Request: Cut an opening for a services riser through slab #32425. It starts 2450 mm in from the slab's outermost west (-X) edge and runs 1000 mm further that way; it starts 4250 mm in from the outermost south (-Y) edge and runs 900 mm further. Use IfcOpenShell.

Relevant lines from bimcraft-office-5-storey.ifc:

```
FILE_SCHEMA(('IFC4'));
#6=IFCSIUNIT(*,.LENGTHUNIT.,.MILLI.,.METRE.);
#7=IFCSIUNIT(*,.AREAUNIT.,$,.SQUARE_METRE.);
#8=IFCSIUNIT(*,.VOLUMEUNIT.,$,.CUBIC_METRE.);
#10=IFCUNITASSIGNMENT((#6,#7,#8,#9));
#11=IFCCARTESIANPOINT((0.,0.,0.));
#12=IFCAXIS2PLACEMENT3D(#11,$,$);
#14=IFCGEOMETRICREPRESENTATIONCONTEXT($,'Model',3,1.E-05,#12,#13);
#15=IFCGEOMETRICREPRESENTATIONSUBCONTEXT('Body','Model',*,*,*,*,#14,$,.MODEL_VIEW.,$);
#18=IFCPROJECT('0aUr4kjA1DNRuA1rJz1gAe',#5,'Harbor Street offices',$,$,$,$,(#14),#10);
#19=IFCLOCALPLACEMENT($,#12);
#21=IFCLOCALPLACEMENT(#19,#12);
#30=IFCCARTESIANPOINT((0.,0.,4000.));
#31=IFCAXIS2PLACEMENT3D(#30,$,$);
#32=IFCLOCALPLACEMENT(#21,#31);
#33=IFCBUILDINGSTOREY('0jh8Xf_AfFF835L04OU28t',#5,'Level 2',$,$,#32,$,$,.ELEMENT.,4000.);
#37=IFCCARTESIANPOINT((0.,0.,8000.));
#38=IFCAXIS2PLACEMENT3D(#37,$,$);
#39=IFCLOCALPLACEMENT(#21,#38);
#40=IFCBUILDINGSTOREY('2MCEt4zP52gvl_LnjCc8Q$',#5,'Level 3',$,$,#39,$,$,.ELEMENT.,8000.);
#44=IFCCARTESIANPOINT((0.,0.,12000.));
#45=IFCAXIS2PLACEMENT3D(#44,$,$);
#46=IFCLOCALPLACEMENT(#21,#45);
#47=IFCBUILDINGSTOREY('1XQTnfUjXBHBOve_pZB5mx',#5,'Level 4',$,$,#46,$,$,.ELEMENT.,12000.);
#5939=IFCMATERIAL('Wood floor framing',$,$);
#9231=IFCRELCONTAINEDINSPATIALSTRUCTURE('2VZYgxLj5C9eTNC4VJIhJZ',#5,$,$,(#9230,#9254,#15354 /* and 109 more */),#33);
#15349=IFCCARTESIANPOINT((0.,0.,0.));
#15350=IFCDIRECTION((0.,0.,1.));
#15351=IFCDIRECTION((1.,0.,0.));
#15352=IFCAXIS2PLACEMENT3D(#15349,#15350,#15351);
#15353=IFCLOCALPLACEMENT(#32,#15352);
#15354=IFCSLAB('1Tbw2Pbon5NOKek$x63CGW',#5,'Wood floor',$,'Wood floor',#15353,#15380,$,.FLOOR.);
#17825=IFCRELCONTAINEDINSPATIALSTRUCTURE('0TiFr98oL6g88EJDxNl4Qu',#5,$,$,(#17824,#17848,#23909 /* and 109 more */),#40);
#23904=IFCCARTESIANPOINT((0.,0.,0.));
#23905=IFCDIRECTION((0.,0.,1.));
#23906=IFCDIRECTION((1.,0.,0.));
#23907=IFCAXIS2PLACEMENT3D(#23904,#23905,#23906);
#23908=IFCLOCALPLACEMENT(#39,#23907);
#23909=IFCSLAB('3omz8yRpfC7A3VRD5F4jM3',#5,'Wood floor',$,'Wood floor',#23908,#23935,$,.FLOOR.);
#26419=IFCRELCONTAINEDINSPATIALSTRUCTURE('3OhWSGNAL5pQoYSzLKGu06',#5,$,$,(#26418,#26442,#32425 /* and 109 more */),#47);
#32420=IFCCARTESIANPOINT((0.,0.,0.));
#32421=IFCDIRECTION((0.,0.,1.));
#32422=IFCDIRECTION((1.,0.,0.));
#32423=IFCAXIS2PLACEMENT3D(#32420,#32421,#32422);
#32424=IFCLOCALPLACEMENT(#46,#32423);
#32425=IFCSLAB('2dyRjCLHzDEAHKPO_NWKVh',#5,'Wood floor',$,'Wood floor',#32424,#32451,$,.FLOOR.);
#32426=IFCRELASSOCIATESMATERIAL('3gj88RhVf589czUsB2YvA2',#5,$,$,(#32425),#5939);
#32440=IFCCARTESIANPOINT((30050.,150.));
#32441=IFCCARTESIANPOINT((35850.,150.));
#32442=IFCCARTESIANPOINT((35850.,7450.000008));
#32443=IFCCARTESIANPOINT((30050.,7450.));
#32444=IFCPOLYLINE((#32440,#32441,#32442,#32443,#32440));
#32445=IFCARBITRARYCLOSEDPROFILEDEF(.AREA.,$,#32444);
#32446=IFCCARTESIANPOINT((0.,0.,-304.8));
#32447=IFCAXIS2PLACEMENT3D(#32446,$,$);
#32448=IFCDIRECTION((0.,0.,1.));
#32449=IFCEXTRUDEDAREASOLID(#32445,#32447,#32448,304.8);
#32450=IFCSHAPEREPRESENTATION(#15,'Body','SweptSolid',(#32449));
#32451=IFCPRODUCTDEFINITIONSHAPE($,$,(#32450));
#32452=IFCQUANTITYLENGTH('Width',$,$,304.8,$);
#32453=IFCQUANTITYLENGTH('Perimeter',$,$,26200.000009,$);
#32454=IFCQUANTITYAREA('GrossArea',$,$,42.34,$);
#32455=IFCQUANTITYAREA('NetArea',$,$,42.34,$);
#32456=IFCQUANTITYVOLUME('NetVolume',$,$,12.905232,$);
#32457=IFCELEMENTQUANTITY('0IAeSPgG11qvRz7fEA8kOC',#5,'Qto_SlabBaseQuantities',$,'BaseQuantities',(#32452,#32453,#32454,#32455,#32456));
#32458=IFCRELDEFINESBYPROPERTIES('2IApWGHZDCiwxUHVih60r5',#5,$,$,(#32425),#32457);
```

```python
import numpy as np
import ifcopenshell
import ifcopenshell.api.feature
import ifcopenshell.api.geometry
import ifcopenshell.api.pset
import ifcopenshell.api.root
import ifcopenshell.geom
import ifcopenshell.util.element
import ifcopenshell.util.placement
import ifcopenshell.util.representation
import ifcopenshell.util.shape
import ifcopenshell.util.unit

model = ifcopenshell.open("bimcraft-office-5-storey.ifc")
unit_scale = ifcopenshell.util.unit.calculate_unit_scale(model)
area_scale = ifcopenshell.util.unit.calculate_unit_scale(model, "AREAUNIT")
volume_scale = ifcopenshell.util.unit.calculate_unit_scale(model, "VOLUMEUNIT")
settings = ifcopenshell.geom.settings()


def volume(element):
    """Net volume in cubic metres, openings subtracted."""
    shape = ifcopenshell.geom.create_shape(settings, element)
    return ifcopenshell.util.shape.get_volume(shape.geometry)


slab = model.by_guid("2dyRjCLHzDEAHKPO_NWKVh")
before = volume(slab)

# Extent in the slab's own axes, in metres. The edges named are its -X and -Y sides.
slab_shape = ifcopenshell.geom.create_shape(settings, slab)
vertices = ifcopenshell.util.shape.get_vertices(slab_shape.geometry)
x_min, y_min, bottom = vertices.min(axis=0)
top = vertices[:, 2].max()

opening = ifcopenshell.api.root.create_entity(model, ifc_class="IfcOpeningElement", name="Services riser opening", predefined_type="OPENING")
context = ifcopenshell.util.representation.get_context(model, "Model", "Body", "MODEL_VIEW")
width, depth = 1, 0.9
outline = [(0.0, 0.0), (width, 0.0), (width, depth), (0.0, depth), (0.0, 0.0)]
# Overshoot both faces by 50 mm so the cut is clean.
shape = ifcopenshell.api.geometry.add_slab_representation(
    model, context=context, depth=top - bottom + 0.1, polyline=outline
)
ifcopenshell.api.geometry.assign_representation(model, product=opening, representation=shape)

matrix = ifcopenshell.util.placement.get_local_placement(slab.ObjectPlacement)
matrix[:, 3] = matrix @ np.append(np.array([x_min + 2.45, y_min + 4.25, bottom - 0.05]) / unit_scale, 1.0)
ifcopenshell.api.geometry.edit_object_placement(model, product=opening, matrix=matrix, is_si=False)
ifcopenshell.api.feature.add_feature(model, feature=opening, element=slab)

after = volume(slab)

# Update the slab's stored quantities.
qto = model.by_id(ifcopenshell.util.element.get_pset(slab, "Qto_SlabBaseQuantities", should_inherit=False)["id"])
ifcopenshell.api.pset.edit_qto(model, qto=qto, properties={
    "NetArea": after / (top - bottom) / area_scale,
    "NetVolume": after / volume_scale,
})

print(f"slab volume {before:.3f} -> {after:.3f} m3")

model.write("bimcraft-office-5-storey_edited.ifc")
```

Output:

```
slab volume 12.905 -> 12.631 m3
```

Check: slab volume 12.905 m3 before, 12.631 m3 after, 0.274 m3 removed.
